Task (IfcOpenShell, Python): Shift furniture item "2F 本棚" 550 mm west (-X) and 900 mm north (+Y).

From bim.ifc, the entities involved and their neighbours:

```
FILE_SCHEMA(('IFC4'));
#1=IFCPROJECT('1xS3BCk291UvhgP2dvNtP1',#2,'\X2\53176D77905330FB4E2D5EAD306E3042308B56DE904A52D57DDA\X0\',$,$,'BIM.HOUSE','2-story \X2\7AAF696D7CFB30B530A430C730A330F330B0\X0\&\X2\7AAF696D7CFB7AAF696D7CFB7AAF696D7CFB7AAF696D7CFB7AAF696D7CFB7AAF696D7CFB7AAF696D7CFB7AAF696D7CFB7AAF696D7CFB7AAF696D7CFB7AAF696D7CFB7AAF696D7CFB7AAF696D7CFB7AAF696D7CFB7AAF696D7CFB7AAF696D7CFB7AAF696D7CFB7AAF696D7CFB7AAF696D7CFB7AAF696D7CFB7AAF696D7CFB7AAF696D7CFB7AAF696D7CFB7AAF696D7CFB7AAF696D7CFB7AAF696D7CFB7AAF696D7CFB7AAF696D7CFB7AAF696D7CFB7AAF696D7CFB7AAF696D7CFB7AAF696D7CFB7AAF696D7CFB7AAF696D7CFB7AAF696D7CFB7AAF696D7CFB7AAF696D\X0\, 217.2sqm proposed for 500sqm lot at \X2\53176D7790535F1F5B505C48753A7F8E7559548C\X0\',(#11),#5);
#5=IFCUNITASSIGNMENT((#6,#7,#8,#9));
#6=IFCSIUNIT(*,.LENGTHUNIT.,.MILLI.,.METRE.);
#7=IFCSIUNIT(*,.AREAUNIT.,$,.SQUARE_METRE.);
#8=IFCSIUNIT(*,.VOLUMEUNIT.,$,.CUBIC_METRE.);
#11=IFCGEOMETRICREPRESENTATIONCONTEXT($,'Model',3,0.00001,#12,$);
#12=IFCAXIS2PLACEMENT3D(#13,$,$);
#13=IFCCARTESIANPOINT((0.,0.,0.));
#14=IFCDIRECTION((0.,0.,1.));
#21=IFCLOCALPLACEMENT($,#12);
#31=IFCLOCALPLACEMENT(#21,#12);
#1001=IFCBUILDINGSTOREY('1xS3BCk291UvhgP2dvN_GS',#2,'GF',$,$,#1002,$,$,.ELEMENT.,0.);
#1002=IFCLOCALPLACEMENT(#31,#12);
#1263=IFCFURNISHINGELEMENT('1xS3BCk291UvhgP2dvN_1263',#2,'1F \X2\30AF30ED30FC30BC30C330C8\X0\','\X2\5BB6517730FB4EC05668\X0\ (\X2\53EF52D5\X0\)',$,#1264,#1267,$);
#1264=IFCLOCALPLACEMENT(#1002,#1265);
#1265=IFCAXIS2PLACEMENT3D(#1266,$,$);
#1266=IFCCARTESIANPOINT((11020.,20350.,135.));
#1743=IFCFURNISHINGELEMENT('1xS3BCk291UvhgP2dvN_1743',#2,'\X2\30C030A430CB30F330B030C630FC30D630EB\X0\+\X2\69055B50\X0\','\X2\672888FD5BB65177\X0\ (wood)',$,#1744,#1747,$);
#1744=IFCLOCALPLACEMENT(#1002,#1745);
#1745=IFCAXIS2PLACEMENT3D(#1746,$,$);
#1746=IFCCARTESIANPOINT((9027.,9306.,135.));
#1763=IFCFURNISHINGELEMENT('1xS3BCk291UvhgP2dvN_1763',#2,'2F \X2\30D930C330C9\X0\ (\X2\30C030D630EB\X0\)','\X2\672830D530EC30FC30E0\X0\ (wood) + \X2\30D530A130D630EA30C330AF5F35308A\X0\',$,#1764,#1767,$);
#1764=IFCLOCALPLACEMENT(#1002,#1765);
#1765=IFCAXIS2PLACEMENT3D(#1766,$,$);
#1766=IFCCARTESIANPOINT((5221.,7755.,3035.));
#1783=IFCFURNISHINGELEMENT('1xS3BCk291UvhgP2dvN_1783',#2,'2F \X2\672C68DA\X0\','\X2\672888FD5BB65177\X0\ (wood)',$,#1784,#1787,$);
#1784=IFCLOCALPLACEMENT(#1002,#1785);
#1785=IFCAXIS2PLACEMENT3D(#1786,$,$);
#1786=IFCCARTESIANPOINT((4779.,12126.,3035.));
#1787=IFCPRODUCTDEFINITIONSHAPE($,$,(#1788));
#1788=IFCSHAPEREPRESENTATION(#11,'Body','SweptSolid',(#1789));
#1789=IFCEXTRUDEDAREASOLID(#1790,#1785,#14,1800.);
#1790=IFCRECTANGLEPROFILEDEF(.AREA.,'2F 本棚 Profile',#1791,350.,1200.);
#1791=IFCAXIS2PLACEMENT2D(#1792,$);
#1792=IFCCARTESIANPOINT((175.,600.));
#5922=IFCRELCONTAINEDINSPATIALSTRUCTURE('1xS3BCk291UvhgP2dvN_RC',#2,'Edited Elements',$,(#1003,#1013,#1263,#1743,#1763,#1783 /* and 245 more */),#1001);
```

```python
import ifcopenshell
import ifcopenshell.api.geometry
import ifcopenshell.util.placement

model = ifcopenshell.open("bim.ifc")

item = model.by_guid("1xS3BCk291UvhgP2dvN_1783")
matrix = ifcopenshell.util.placement.get_local_placement(item.ObjectPlacement)
matrix[0, 3] -= 550.0
matrix[1, 3] += 900.0
ifcopenshell.api.geometry.edit_object_placement(model, product=item, matrix=matrix, is_si=False)

print(ifcopenshell.util.placement.get_local_placement(item.ObjectPlacement).round(3) + 0.0)

model.write("bim_updated.ifc")
```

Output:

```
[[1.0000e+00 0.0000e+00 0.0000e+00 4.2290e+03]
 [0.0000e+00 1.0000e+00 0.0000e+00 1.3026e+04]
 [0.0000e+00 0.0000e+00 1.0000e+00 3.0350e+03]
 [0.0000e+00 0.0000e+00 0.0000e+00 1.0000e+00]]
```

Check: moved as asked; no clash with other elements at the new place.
